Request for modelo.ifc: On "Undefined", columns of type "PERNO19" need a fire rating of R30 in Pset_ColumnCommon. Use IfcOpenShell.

First a look at what the model holds.

```python
import ifcopenshell
import ifcopenshell.util.element

model = ifcopenshell.open("modelo.ifc")
print(model.schema)
storey = next(s for s in model.by_type("IfcBuildingStorey") if s.Name == "Undefined")
columns = [e for e in ifcopenshell.util.element.get_decomposition(storey) if e.is_a("IfcColumn")]
seen = {}
for e in columns:
    element_type = ifcopenshell.util.element.get_type(e)
    key = (element_type.Name if element_type != e and element_type else None, ifcopenshell.util.element.get_pset(e, "Pset_ColumnCommon", "FireRating"))
    seen[key] = seen.get(key, 0) + 1
for (name, value), count in sorted(seen.items(), key=str):
    print(count, "x", name, "|", value)
```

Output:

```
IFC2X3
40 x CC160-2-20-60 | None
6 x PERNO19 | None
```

```python
import ifcopenshell
import ifcopenshell.api.pset
import ifcopenshell.util.element

model = ifcopenshell.open("modelo.ifc")

storey = next(s for s in model.by_type("IfcBuildingStorey") if s.Name == "Undefined")
columns = [e for e in ifcopenshell.util.element.get_decomposition(storey) if e.is_a("IfcColumn")]

count = 0
for e in columns:
    element_type = ifcopenshell.util.element.get_type(e)
    if element_type in (None, e) or element_type.Name != "PERNO19":
        continue
    found = ifcopenshell.util.element.get_pset(e, "Pset_ColumnCommon", should_inherit=False)
    if found:
        pset = model.by_id(found["id"])
        if len(ifcopenshell.util.element.get_elements_by_pset(pset)) > 1:
            pset = ifcopenshell.api.pset.unshare_pset(model, products=[e], pset=pset)[0]
    else:
        pset = ifcopenshell.api.pset.add_pset(model, product=e, name="Pset_ColumnCommon")
    ifcopenshell.api.pset.edit_pset(model, pset=pset, properties={"FireRating": "R30"})
    count += 1

print(count, "columns updated")

model.write("modelo_updated.ifc")
```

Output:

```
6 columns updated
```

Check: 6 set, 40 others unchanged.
